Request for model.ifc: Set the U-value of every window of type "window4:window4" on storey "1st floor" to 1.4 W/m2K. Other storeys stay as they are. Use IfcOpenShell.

First a look at what the model holds.

```python
import ifcopenshell
import ifcopenshell.util.element

model = ifcopenshell.open("model.ifc")
print(model.schema)
storey = next(s for s in model.by_type("IfcBuildingStorey") if s.Name == "1st floor")
windows = [e for e in ifcopenshell.util.element.get_decomposition(storey) if e.is_a("IfcWindow")]
seen = {}
for e in windows:
    element_type = ifcopenshell.util.element.get_type(e)
    key = (element_type.Name if element_type != e and element_type else None, ifcopenshell.util.element.get_pset(e, "Pset_WindowCommon", "ThermalTransmittance"))
    seen[key] = seen.get(key, 0) + 1
for (name, value), count in sorted(seen.items(), key=str):
    print(count, "x", name, "|", value)
```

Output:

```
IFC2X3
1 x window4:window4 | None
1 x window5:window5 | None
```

```python
import ifcopenshell
import ifcopenshell.api.pset
import ifcopenshell.util.element

model = ifcopenshell.open("model.ifc")

storey = next(s for s in model.by_type("IfcBuildingStorey") if s.Name == "1st floor")
windows = [e for e in ifcopenshell.util.element.get_decomposition(storey) if e.is_a("IfcWindow")]

count = 0
for e in windows:
    element_type = ifcopenshell.util.element.get_type(e)
    if element_type in (None, e) or element_type.Name != "window4:window4":
        continue
    # add_pset returns the element's existing set when there is one.
    pset = ifcopenshell.api.pset.add_pset(model, product=e, name="Pset_WindowCommon")
    ifcopenshell.api.pset.edit_pset(model, pset=pset, properties={"ThermalTransmittance": 1.4})
    count += 1

print(count, "windows updated")

model.write("model_updated.ifc")
```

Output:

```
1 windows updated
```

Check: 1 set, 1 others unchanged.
